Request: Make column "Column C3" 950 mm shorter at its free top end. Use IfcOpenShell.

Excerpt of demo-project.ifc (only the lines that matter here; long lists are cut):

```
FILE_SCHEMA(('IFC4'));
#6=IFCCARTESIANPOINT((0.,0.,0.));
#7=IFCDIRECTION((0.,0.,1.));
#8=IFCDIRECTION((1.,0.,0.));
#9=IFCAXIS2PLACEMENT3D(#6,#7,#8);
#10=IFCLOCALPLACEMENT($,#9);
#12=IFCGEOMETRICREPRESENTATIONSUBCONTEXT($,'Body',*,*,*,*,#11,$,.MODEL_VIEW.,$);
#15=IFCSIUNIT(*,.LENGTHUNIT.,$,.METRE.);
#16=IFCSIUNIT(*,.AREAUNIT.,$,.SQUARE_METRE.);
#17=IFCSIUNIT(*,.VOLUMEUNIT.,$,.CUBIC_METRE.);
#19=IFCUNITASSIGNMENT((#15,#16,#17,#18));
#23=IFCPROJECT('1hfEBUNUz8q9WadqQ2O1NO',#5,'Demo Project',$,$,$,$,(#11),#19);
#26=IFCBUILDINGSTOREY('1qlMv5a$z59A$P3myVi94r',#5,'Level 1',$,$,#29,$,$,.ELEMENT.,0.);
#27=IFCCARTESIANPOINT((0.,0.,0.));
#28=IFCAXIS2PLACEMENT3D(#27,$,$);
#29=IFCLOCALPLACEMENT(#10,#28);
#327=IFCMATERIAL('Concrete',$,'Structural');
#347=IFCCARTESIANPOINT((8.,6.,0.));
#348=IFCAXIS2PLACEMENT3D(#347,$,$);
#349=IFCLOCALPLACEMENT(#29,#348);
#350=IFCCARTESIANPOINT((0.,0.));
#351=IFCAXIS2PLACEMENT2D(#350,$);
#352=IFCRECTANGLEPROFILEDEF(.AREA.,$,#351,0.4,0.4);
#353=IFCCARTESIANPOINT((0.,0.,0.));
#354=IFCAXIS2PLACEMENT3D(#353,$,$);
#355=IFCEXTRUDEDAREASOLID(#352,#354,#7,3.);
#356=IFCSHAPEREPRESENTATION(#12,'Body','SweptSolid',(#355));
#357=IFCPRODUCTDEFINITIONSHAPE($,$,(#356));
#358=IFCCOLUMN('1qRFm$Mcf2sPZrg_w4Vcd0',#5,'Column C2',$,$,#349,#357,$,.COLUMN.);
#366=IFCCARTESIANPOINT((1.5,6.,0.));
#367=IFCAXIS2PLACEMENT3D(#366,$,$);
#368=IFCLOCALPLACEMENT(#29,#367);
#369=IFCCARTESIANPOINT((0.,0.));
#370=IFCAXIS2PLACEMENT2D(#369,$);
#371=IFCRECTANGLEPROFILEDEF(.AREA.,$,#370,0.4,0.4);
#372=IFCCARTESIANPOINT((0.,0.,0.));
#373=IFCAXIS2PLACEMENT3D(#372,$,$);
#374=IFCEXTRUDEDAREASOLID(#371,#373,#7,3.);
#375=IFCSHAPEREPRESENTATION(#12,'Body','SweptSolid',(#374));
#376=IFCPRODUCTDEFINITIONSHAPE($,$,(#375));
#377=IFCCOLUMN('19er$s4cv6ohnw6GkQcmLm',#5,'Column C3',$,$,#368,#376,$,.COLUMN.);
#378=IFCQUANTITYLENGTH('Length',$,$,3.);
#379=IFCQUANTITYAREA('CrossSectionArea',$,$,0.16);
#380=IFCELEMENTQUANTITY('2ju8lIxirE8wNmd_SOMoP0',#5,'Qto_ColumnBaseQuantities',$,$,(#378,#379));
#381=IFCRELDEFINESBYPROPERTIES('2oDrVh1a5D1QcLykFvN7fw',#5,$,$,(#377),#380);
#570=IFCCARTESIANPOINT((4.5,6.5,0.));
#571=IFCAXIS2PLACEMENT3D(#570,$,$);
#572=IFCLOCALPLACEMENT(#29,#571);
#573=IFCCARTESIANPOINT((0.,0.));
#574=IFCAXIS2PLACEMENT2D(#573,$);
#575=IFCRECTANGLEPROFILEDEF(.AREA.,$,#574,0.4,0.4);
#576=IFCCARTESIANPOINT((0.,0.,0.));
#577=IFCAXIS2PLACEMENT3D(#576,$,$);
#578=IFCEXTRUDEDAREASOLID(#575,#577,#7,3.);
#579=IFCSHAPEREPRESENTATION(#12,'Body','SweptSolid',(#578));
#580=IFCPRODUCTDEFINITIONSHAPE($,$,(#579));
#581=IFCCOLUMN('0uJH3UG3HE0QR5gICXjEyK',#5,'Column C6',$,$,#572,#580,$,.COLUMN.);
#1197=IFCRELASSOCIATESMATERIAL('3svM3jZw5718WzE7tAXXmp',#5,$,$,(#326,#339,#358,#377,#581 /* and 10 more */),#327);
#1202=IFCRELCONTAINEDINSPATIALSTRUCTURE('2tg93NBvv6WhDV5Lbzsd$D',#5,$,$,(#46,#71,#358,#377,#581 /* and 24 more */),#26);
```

```python
import ifcopenshell
import ifcopenshell.api.pset
import ifcopenshell.util.element
import ifcopenshell.util.unit

model = ifcopenshell.open("demo-project.ifc")
unit_scale = ifcopenshell.util.unit.calculate_unit_scale(model)

member = model.by_id(377)
change = -0.95 / unit_scale

# The extrusion runs towards the end named, so only its depth changes.
body = next(r for r in member.Representation.Representations if r.RepresentationIdentifier == "Body")
solid = body.Items[0]
old_length = solid.Depth
solid.Depth += change

# Update the stored length and volume.
qto = model.by_id(ifcopenshell.util.element.get_pset(member, "Qto_ColumnBaseQuantities", should_inherit=False)["id"])
ifcopenshell.api.pset.edit_qto(model, qto=qto, properties={"Length": solid.Depth})

print(f"length {old_length:g} -> {solid.Depth:g}")

model.write("demo-project_v2.ifc")
```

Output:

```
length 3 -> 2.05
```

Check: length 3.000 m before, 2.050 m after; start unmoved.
